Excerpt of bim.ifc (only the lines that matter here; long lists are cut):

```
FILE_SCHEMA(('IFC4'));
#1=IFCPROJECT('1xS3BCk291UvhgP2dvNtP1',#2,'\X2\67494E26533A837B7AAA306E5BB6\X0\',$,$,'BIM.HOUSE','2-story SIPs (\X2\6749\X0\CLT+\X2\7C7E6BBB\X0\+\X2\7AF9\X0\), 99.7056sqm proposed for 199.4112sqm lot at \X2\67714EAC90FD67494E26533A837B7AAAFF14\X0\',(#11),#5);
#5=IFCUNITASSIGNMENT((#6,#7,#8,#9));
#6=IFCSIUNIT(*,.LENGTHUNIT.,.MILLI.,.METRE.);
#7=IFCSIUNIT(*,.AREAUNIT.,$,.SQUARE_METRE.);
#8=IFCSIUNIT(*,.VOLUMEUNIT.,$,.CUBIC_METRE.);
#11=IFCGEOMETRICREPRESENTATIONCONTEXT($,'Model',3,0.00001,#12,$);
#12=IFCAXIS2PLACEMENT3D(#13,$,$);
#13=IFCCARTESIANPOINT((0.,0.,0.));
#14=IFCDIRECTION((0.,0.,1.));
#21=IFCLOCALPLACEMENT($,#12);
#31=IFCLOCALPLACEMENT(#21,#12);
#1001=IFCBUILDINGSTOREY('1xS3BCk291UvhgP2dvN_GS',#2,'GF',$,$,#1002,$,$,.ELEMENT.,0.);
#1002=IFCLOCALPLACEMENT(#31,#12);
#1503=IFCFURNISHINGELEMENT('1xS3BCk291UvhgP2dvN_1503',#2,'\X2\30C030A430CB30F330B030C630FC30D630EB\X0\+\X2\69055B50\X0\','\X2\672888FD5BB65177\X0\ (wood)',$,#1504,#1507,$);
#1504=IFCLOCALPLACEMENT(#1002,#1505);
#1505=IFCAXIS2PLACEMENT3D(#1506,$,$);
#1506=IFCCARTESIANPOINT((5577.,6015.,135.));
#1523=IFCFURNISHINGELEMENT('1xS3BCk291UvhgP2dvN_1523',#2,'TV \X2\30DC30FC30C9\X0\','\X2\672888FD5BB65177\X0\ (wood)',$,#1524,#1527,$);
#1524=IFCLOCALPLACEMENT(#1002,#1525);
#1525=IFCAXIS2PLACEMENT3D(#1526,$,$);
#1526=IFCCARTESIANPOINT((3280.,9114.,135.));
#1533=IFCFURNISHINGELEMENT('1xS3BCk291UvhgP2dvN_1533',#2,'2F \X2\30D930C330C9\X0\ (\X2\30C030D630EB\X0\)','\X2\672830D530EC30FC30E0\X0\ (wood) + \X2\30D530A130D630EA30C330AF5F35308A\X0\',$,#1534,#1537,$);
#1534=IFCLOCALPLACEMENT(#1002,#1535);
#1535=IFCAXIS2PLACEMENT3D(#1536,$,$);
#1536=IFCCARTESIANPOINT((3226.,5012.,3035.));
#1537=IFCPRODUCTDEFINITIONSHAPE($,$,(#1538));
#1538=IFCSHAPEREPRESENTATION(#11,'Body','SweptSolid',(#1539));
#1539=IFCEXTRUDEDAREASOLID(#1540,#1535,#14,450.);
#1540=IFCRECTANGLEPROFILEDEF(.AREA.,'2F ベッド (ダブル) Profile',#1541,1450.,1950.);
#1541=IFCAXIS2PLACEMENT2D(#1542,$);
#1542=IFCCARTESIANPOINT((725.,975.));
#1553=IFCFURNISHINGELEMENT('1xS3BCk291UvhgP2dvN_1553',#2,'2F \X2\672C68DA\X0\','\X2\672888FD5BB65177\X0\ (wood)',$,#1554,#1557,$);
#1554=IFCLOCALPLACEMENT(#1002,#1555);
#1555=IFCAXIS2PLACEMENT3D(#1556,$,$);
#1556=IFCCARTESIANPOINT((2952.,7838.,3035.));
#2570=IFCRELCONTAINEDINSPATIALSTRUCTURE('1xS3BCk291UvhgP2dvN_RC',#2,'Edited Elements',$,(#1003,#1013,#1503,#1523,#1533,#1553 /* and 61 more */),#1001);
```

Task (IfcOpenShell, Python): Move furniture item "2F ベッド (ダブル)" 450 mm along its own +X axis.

```python
import ifcopenshell
import ifcopenshell.api.geometry
import ifcopenshell.util.placement
import ifcopenshell.util.unit

model = ifcopenshell.open("bim.ifc")
unit_scale = ifcopenshell.util.unit.calculate_unit_scale(model)

item = model.by_id(1533)
matrix = ifcopenshell.util.placement.get_local_placement(item.ObjectPlacement)
matrix[:3, 3] += matrix[:3, 0] * 0.45 / unit_scale
ifcopenshell.api.geometry.edit_object_placement(model, product=item, matrix=matrix, is_si=False)

print(ifcopenshell.util.placement.get_local_placement(item.ObjectPlacement).round(3) + 0.0)

model.write("bim_rev.ifc")
```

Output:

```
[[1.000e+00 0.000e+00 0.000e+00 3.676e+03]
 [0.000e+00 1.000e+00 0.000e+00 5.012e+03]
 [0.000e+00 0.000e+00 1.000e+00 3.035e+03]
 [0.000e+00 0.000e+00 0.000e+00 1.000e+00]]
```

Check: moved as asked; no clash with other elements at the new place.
